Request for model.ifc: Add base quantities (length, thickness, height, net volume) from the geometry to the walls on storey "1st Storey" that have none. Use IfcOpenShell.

First a look at what the model holds.

```python
import ifcopenshell
import ifcopenshell.util.element
import ifcopenshell.util.unit

model = ifcopenshell.open("model.ifc")
print(model.schema)
for unit_type in ("LENGTHUNIT", "AREAUNIT", "VOLUMEUNIT"):
    print(unit_type, ifcopenshell.util.unit.calculate_unit_scale(model, unit_type))
storey = next(s for s in model.by_type("IfcBuildingStorey") if s.Name == "1st Storey")
walls = [e for e in ifcopenshell.util.element.get_decomposition(storey) if e.is_a("IfcWall")]
for e in sorted(walls, key=lambda e: e.id()):
    print(e.id(), e.is_a(), e.Name, list(ifcopenshell.util.element.get_psets(e, qtos_only=True)), sep=" | ")
```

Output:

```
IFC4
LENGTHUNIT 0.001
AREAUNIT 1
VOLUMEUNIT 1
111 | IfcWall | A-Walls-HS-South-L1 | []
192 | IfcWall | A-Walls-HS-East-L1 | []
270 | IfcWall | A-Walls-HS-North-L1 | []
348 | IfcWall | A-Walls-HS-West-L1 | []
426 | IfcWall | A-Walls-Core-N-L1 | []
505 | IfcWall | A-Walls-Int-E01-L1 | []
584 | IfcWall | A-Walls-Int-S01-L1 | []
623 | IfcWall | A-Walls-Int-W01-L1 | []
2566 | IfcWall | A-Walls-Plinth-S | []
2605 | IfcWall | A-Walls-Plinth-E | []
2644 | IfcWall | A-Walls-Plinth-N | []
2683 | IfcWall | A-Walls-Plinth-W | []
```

```python
import ifcopenshell
import ifcopenshell.api.pset
import ifcopenshell.geom
import ifcopenshell.util.element
import ifcopenshell.util.shape
import ifcopenshell.util.unit

model = ifcopenshell.open("model.ifc")
unit_scale = ifcopenshell.util.unit.calculate_unit_scale(model)
volume_scale = ifcopenshell.util.unit.calculate_unit_scale(model, "VOLUMEUNIT")
settings = ifcopenshell.geom.settings()

storey = next(s for s in model.by_type("IfcBuildingStorey") if s.Name == "1st Storey")
walls = [e for e in ifcopenshell.util.element.get_decomposition(storey) if e.is_a("IfcWall")]

for e in sorted(walls, key=lambda e: e.id()):
    if ifcopenshell.util.element.get_psets(e, qtos_only=True, should_inherit=False):
        continue
    # Geometry comes back in metres, in the element's own axes.
    shape = ifcopenshell.geom.create_shape(settings, e)
    values = {
        "Length": ifcopenshell.util.shape.get_x(shape.geometry) / unit_scale,
        "Width": ifcopenshell.util.shape.get_y(shape.geometry) / unit_scale,
        "Height": ifcopenshell.util.shape.get_z(shape.geometry) / unit_scale,
        "NetVolume": ifcopenshell.util.shape.get_volume(shape.geometry) / volume_scale,
    }
    qto = ifcopenshell.api.pset.add_qto(model, product=e, name="Qto_WallBaseQuantities")
    ifcopenshell.api.pset.edit_qto(model, qto=qto, properties=values)
    print(e.id(), {k: round(v, 3) for k, v in values.items()})

model.write("model-out.ifc")
```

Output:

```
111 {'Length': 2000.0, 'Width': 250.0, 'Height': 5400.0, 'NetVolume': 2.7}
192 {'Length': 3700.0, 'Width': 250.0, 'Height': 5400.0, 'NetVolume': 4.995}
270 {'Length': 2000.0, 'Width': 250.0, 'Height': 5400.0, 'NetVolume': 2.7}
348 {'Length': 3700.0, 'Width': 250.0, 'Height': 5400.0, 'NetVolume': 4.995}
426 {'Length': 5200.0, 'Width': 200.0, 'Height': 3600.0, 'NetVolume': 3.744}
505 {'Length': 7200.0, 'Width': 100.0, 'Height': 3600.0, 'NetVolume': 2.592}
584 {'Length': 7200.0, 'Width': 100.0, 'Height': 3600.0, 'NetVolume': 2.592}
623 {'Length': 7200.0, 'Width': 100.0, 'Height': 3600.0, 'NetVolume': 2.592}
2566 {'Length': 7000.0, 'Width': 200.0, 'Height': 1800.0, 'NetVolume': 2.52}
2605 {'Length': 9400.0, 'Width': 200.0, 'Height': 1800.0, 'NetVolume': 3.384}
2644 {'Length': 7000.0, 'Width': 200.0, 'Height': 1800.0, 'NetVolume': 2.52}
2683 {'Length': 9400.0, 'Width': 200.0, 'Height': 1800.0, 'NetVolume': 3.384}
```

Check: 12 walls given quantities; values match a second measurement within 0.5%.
